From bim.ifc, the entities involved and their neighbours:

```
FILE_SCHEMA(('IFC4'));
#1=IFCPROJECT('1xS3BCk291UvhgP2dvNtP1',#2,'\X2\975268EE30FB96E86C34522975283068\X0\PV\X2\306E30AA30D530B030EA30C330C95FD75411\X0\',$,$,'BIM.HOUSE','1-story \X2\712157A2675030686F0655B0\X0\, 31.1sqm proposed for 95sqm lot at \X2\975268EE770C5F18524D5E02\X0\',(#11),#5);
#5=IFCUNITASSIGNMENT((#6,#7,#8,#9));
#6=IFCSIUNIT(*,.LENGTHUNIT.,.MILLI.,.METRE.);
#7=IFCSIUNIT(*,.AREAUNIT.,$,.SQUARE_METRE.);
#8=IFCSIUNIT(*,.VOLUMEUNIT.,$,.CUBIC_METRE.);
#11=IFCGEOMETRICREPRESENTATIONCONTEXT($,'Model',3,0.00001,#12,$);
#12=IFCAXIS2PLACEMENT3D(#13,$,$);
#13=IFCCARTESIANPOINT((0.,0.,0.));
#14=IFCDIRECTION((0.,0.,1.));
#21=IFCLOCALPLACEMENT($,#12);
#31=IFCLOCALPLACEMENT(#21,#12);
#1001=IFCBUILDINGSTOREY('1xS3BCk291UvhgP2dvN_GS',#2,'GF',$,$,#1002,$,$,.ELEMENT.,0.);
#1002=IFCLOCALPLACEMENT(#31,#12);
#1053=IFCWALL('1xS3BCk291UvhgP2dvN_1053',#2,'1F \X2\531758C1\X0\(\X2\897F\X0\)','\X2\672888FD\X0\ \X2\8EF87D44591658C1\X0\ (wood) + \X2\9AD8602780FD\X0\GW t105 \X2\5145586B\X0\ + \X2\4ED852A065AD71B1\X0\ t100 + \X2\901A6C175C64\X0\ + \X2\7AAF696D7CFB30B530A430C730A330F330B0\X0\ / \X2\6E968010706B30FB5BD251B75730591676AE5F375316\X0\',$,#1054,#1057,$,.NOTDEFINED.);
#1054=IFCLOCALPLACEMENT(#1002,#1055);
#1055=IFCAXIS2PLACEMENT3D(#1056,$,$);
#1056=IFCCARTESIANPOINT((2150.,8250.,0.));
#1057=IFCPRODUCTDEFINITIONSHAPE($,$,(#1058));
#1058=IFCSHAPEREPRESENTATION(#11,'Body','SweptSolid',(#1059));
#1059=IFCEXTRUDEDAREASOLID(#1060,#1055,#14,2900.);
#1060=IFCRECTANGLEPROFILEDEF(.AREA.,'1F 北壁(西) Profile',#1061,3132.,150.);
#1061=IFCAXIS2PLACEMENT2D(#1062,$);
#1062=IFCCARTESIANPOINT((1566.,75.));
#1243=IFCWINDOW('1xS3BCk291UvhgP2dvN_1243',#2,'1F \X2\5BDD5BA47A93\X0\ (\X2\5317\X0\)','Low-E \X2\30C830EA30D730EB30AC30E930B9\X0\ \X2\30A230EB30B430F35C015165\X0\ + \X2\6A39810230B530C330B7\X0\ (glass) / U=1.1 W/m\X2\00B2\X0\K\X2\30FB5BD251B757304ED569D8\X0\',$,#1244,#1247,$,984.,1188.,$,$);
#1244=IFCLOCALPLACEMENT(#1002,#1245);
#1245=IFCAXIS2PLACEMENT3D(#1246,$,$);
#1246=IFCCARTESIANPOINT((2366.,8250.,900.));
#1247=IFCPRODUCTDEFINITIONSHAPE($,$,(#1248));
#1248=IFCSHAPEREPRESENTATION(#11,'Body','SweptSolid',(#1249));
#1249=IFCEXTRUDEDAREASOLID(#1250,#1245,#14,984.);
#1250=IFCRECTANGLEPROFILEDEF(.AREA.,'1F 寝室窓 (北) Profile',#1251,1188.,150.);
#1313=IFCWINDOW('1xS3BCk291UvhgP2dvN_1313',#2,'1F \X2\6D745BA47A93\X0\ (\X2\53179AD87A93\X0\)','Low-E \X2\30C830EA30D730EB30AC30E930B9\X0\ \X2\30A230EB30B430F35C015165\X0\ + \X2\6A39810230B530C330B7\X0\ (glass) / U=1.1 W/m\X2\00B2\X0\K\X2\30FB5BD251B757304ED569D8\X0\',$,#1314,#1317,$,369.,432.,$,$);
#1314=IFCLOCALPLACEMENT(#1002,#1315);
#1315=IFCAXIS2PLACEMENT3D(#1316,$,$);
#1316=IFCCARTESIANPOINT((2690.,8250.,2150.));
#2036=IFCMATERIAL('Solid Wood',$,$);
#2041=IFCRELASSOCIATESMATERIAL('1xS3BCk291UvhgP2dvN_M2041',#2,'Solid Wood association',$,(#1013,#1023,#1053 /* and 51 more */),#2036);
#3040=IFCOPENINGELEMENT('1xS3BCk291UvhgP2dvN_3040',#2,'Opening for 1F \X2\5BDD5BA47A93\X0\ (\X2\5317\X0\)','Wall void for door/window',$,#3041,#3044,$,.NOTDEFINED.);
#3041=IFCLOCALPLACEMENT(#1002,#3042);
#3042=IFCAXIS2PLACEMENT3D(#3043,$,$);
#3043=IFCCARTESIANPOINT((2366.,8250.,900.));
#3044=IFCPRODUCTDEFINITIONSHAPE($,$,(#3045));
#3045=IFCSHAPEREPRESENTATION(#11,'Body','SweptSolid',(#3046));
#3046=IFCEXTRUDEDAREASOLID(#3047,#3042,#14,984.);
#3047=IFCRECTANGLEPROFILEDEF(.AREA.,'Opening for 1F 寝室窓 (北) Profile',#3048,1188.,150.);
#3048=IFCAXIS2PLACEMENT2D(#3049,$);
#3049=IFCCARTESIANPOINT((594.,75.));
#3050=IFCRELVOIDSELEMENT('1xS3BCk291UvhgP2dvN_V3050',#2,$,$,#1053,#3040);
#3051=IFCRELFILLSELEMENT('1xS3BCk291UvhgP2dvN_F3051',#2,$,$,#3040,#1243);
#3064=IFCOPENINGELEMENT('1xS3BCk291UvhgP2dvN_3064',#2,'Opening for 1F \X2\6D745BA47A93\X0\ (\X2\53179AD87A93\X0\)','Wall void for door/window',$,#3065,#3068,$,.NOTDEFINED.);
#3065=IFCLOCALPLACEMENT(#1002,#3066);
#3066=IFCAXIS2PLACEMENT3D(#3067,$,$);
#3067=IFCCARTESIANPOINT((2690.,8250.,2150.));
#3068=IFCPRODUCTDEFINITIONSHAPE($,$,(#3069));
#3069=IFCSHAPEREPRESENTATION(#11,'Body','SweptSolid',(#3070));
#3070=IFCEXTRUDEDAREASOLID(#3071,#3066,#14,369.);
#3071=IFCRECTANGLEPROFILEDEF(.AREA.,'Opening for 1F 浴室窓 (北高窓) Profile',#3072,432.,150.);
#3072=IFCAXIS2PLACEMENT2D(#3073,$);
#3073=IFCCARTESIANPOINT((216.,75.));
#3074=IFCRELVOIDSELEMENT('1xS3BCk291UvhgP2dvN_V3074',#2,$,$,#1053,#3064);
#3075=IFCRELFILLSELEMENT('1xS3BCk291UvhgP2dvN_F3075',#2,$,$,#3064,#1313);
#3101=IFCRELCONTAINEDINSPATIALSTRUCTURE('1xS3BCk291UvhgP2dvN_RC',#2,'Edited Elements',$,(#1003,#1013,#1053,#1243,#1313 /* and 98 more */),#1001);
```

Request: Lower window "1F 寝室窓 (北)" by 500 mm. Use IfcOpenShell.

```python
import numpy as np
import ifcopenshell
import ifcopenshell.api.geometry
import ifcopenshell.util.placement
import ifcopenshell.util.unit

model = ifcopenshell.open("bim.ifc")
unit_scale = ifcopenshell.util.unit.calculate_unit_scale(model)

window = model.by_guid("1xS3BCk291UvhgP2dvN_1243")
opening = window.FillsVoids[0].RelatingOpeningElement
dz = -0.5 / unit_scale

shift = np.array([0.0, 0.0, dz])
# The window is not placed relative to its opening, so move both.
for product in (opening, window):
    matrix = ifcopenshell.util.placement.get_local_placement(product.ObjectPlacement)
    matrix[:3, 3] += shift
    ifcopenshell.api.geometry.edit_object_placement(model, product=product, matrix=matrix, is_si=False)

print(f"moved by {dz * unit_scale:+.3f} m")

model.write("bim_updated.ifc")
```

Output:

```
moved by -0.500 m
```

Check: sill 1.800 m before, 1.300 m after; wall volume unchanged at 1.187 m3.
